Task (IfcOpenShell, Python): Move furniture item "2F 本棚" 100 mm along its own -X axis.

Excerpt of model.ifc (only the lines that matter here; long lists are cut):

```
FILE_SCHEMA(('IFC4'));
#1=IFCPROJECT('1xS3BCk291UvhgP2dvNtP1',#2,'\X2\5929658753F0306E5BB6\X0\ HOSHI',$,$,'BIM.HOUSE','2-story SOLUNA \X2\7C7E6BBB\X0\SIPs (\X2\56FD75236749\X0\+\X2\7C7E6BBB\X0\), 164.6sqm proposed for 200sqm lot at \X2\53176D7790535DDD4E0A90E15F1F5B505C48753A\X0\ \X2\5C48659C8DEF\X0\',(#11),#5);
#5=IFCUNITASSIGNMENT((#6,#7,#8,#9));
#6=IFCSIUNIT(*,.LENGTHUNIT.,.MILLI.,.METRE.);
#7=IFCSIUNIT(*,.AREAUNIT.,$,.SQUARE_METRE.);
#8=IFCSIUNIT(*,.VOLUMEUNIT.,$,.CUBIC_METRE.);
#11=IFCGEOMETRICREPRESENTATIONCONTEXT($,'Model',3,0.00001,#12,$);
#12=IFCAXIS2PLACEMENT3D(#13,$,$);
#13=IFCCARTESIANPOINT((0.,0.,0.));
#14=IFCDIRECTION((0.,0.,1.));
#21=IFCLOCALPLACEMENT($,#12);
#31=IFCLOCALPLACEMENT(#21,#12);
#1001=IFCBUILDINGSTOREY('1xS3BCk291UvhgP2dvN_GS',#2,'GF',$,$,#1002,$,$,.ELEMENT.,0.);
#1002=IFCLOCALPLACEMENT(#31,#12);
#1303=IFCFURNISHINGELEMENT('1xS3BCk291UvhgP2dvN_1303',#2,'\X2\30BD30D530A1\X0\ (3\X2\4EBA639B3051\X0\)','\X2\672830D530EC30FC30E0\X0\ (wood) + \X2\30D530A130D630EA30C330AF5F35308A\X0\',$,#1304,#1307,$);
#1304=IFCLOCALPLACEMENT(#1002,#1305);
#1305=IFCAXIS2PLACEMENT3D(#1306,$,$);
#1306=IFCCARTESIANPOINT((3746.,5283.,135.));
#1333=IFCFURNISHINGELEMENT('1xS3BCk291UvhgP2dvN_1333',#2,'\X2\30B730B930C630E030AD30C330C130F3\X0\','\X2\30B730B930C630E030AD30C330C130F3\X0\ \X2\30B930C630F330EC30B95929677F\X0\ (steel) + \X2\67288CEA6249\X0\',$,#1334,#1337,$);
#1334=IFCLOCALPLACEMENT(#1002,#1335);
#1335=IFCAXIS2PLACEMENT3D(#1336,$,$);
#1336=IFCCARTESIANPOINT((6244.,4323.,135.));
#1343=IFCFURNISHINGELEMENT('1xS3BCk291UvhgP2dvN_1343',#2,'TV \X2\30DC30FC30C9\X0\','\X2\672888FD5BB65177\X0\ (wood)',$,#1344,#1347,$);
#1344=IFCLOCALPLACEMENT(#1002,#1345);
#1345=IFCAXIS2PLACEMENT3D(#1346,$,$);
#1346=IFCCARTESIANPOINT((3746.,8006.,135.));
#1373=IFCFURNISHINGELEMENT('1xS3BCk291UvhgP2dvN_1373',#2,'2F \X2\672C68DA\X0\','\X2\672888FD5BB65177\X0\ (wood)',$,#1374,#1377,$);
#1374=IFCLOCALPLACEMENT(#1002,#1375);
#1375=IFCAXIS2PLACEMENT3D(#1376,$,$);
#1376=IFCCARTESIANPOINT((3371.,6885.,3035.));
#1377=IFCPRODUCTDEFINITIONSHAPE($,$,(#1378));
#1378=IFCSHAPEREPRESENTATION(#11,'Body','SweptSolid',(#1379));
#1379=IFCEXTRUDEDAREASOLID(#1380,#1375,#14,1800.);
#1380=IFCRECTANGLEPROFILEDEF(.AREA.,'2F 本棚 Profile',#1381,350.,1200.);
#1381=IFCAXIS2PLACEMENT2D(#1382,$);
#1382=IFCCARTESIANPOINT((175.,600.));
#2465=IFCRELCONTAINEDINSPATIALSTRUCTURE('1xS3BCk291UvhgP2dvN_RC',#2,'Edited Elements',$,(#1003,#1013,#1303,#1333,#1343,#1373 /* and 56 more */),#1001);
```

```python
import ifcopenshell
import ifcopenshell.api.geometry
import ifcopenshell.util.placement

model = ifcopenshell.open("model.ifc")

item = model.by_guid("1xS3BCk291UvhgP2dvN_1373")
matrix = ifcopenshell.util.placement.get_local_placement(item.ObjectPlacement)
matrix[:3, 3] -= matrix[:3, 0] * 100.0
ifcopenshell.api.geometry.edit_object_placement(model, product=item, matrix=matrix, is_si=False)

print(ifcopenshell.util.placement.get_local_placement(item.ObjectPlacement).round(3) + 0.0)

model.write("model_rev.ifc")
```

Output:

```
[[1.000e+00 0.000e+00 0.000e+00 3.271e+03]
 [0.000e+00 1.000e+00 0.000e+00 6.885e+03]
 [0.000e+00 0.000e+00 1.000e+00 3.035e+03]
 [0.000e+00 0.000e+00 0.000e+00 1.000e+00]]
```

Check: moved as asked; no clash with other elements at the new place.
